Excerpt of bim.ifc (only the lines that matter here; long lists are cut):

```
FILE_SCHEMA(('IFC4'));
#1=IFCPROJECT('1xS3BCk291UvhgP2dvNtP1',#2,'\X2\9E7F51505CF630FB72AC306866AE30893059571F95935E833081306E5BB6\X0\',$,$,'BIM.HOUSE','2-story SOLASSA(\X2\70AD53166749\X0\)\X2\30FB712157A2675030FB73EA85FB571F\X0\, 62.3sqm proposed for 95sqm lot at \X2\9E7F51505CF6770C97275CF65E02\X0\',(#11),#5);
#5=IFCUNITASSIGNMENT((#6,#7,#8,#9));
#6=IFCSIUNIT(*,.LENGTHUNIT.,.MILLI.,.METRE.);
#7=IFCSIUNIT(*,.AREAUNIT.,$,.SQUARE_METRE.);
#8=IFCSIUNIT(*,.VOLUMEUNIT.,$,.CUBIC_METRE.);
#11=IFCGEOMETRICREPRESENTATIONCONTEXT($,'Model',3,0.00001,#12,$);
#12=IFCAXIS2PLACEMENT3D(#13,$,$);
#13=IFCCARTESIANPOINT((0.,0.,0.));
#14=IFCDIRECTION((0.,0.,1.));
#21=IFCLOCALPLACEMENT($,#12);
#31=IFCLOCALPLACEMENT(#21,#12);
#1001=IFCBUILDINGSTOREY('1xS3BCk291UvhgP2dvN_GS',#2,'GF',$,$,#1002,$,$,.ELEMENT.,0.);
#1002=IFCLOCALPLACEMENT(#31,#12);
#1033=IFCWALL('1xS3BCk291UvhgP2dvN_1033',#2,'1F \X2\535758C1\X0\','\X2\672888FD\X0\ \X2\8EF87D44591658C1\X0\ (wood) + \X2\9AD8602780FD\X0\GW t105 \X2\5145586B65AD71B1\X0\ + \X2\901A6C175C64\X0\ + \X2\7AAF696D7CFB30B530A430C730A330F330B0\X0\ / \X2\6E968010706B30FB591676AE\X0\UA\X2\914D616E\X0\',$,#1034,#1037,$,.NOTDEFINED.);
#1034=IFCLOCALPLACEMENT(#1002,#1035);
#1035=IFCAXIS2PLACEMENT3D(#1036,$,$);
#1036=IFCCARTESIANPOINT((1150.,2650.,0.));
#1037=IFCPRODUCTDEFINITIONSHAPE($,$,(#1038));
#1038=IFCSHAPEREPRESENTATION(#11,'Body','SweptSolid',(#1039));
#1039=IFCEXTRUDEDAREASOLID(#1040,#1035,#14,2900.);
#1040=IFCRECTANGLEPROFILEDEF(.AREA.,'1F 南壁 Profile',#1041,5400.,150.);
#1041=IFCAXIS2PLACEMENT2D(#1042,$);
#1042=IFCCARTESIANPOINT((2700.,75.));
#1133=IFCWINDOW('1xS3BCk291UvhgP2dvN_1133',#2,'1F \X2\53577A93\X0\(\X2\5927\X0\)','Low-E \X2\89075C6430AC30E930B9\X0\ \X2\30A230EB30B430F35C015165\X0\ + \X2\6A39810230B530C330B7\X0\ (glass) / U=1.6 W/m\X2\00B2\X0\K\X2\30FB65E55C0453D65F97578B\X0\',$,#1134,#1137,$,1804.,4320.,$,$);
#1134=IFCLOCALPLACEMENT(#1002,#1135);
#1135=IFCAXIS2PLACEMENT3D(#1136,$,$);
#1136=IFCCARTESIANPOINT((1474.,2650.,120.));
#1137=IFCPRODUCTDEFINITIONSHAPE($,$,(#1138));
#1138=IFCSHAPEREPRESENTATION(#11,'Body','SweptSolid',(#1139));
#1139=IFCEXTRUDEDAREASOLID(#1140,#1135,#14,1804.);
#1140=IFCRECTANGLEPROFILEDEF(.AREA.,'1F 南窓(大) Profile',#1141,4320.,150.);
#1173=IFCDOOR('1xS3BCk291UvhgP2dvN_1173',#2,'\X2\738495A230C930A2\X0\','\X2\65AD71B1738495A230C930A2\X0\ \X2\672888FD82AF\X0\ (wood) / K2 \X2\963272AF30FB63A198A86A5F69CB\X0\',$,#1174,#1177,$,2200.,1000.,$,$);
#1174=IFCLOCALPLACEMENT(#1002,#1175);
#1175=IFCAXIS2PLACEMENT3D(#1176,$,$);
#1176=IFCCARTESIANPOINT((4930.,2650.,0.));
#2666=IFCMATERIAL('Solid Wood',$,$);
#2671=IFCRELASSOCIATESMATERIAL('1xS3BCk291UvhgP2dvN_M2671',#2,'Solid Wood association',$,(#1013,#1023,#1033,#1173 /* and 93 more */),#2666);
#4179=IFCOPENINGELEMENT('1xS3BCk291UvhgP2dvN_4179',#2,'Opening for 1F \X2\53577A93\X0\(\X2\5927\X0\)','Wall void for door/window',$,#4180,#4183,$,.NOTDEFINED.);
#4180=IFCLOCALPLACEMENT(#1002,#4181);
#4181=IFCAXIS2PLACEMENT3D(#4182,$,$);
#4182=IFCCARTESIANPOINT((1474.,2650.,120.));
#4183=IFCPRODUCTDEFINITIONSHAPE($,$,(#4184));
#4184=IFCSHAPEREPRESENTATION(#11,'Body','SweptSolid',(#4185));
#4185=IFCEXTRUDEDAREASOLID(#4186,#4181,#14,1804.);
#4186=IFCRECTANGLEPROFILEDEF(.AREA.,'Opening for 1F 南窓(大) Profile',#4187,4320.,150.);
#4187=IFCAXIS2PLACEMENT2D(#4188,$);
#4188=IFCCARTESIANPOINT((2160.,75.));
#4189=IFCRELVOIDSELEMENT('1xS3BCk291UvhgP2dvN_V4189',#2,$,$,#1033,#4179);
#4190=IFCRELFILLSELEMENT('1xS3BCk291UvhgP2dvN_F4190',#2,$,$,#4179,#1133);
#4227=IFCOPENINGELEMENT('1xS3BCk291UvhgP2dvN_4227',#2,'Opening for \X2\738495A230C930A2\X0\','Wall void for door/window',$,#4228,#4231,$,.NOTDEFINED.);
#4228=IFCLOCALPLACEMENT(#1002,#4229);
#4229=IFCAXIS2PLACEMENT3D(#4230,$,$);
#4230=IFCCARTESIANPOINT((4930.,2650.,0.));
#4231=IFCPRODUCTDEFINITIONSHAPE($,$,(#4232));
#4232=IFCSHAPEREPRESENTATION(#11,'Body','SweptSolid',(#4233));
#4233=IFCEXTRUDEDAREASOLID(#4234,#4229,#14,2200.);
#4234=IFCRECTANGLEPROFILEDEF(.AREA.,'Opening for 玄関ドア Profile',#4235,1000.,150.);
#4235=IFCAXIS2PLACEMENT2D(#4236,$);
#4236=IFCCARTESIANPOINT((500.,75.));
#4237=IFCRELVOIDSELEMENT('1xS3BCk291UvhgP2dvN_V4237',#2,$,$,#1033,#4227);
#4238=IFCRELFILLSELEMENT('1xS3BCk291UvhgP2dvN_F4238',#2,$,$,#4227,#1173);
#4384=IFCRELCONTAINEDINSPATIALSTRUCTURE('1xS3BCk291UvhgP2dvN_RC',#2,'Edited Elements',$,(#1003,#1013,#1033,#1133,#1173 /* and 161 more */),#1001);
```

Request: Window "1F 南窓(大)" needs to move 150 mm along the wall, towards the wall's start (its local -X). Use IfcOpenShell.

```python
import ifcopenshell
import ifcopenshell.api.geometry
import ifcopenshell.util.placement
import ifcopenshell.util.unit

model = ifcopenshell.open("bim.ifc")
unit_scale = ifcopenshell.util.unit.calculate_unit_scale(model)

window = model.by_guid("1xS3BCk291UvhgP2dvN_1133")
opening = window.FillsVoids[0].RelatingOpeningElement
wall = opening.VoidsElements[0].RelatingBuildingElement

wall_matrix = ifcopenshell.util.placement.get_local_placement(wall.ObjectPlacement)
shift = wall_matrix[:3, 0] * -0.15 / unit_scale
before = ifcopenshell.util.placement.get_local_placement(window.ObjectPlacement)[:3, 3].copy()

# The window is not placed relative to its opening, so move both.
for product in (opening, window):
    matrix = ifcopenshell.util.placement.get_local_placement(product.ObjectPlacement)
    matrix[:3, 3] += shift
    ifcopenshell.api.geometry.edit_object_placement(model, product=product, matrix=matrix, is_si=False)

after = ifcopenshell.util.placement.get_local_placement(window.ObjectPlacement)[:3, 3]
print("window moved by", (after - before).round(3) + 0.0)

model.write("bim_rev.ifc")
```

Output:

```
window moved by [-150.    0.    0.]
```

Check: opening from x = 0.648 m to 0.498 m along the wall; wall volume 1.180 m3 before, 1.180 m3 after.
